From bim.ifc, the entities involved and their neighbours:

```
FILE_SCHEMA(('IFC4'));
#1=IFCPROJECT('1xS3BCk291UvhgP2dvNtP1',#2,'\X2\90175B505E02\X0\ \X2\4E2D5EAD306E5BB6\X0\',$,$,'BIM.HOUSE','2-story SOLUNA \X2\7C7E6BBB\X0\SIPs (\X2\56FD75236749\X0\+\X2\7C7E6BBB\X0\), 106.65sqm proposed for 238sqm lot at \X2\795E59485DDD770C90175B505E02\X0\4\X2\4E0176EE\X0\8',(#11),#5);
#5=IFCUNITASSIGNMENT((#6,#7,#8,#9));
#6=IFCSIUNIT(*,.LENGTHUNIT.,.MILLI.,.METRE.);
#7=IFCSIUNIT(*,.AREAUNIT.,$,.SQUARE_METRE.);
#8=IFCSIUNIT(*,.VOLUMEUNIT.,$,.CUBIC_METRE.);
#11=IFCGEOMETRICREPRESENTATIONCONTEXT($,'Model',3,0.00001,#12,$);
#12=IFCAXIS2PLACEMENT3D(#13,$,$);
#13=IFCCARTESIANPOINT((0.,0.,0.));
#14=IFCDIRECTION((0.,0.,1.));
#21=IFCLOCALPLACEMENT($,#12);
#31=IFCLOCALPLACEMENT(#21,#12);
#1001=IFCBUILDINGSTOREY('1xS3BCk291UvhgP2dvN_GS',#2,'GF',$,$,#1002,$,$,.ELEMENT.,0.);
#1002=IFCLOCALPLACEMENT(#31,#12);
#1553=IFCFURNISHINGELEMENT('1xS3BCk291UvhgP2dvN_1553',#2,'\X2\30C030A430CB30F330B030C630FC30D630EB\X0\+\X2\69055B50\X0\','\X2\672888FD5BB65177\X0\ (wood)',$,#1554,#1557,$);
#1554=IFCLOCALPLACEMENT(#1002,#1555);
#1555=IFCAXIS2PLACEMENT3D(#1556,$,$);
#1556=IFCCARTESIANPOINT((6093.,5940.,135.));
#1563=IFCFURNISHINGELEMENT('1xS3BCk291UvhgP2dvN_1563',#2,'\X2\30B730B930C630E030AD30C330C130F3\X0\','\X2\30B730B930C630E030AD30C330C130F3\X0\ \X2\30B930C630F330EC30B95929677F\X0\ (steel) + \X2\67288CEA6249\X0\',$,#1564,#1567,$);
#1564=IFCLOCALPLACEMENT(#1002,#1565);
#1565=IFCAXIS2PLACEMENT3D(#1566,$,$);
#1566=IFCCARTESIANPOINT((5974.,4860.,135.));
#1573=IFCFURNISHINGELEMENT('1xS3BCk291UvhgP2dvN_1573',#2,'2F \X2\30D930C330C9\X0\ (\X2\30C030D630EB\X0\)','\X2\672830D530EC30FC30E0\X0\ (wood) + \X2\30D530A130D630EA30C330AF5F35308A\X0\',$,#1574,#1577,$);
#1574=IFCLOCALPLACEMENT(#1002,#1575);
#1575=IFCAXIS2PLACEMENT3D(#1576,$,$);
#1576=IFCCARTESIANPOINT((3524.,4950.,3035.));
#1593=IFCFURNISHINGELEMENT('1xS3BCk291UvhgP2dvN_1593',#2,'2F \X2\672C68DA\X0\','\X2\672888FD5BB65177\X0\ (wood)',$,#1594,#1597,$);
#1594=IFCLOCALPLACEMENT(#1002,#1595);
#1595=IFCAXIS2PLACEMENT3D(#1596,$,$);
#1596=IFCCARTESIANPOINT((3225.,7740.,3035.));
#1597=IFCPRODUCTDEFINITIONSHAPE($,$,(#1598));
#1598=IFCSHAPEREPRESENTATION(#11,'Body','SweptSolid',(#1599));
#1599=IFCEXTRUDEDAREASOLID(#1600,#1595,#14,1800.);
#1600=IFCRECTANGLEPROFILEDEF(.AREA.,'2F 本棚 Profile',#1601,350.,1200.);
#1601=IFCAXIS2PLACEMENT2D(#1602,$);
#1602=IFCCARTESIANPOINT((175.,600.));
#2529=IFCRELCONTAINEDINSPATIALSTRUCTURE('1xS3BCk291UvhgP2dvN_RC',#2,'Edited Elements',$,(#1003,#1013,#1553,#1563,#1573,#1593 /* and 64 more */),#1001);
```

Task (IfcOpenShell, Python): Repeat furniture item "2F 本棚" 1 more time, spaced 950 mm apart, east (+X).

```python
import numpy as np
import ifcopenshell
import ifcopenshell.api.geometry
import ifcopenshell.api.root
import ifcopenshell.util.element
import ifcopenshell.util.placement
import ifcopenshell.util.unit

model = ifcopenshell.open("bim.ifc")
unit_scale = ifcopenshell.util.unit.calculate_unit_scale(model)


def reuse_history(source, copy):
    """copy_class also copies each property set's owner history, people and application; keep the originals."""
    for rel in copy.IsDefinedBy:
        if rel.is_a("IfcRelDefinesByProperties") and (history := rel.RelatingPropertyDefinition.OwnerHistory):
            rel.RelatingPropertyDefinition.OwnerHistory = source.OwnerHistory
            ifcopenshell.util.element.remove_deep2(model, history)


source = model.by_guid("1xS3BCk291UvhgP2dvN_1593")
base = ifcopenshell.util.placement.get_local_placement(source.ObjectPlacement)
step = np.array([1.0, 0.0, 0.0]) * 0.95 / unit_scale

for i in range(1, 2):
    copy = ifcopenshell.api.root.copy_class(model, product=source)
    copy.Representation = ifcopenshell.util.element.copy_deep(
        model, source.Representation, exclude=["IfcGeometricRepresentationContext", "IfcRepresentationMap"]
    )
    reuse_history(source, copy)
    matrix = base.copy()
    matrix[:3, 3] += i * step
    print("added at", matrix[:3, 3].round(3) + 0.0)
    ifcopenshell.api.geometry.edit_object_placement(model, product=copy, matrix=matrix, is_si=False)

model.write("bim_rev.ifc")
```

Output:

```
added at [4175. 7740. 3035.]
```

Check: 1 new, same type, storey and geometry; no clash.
